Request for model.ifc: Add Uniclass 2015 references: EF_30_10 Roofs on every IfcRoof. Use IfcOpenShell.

First a look at what the model holds.

```python
import ifcopenshell

model = ifcopenshell.open("model.ifc")
print(model.schema)
print("classifications:", [c.Name for c in model.by_type("IfcClassification")])
for ifc_class in ("IfcDoor", "IfcRoof", "IfcStair", "IfcWall", "IfcWindow"):
    print(ifc_class, len(model.by_type(ifc_class)))
```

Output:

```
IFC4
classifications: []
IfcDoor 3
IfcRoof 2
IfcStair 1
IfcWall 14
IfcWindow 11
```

```python
import ifcopenshell
import ifcopenshell.api.classification

model = ifcopenshell.open("model.ifc")

system = ifcopenshell.api.classification.add_classification(model, classification="Uniclass 2015")

codes = {
    "IfcRoof": ("EF_30_10", "Roofs"),
}
for ifc_class, (code, name) in codes.items():
    products = model.by_type(ifc_class)
    ifcopenshell.api.classification.add_reference(
        model, products=products, classification=system, identification=code, name=name
    )
    print(code, len(products))

model.write("model_edited.ifc")
```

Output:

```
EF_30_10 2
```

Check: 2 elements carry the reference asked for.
